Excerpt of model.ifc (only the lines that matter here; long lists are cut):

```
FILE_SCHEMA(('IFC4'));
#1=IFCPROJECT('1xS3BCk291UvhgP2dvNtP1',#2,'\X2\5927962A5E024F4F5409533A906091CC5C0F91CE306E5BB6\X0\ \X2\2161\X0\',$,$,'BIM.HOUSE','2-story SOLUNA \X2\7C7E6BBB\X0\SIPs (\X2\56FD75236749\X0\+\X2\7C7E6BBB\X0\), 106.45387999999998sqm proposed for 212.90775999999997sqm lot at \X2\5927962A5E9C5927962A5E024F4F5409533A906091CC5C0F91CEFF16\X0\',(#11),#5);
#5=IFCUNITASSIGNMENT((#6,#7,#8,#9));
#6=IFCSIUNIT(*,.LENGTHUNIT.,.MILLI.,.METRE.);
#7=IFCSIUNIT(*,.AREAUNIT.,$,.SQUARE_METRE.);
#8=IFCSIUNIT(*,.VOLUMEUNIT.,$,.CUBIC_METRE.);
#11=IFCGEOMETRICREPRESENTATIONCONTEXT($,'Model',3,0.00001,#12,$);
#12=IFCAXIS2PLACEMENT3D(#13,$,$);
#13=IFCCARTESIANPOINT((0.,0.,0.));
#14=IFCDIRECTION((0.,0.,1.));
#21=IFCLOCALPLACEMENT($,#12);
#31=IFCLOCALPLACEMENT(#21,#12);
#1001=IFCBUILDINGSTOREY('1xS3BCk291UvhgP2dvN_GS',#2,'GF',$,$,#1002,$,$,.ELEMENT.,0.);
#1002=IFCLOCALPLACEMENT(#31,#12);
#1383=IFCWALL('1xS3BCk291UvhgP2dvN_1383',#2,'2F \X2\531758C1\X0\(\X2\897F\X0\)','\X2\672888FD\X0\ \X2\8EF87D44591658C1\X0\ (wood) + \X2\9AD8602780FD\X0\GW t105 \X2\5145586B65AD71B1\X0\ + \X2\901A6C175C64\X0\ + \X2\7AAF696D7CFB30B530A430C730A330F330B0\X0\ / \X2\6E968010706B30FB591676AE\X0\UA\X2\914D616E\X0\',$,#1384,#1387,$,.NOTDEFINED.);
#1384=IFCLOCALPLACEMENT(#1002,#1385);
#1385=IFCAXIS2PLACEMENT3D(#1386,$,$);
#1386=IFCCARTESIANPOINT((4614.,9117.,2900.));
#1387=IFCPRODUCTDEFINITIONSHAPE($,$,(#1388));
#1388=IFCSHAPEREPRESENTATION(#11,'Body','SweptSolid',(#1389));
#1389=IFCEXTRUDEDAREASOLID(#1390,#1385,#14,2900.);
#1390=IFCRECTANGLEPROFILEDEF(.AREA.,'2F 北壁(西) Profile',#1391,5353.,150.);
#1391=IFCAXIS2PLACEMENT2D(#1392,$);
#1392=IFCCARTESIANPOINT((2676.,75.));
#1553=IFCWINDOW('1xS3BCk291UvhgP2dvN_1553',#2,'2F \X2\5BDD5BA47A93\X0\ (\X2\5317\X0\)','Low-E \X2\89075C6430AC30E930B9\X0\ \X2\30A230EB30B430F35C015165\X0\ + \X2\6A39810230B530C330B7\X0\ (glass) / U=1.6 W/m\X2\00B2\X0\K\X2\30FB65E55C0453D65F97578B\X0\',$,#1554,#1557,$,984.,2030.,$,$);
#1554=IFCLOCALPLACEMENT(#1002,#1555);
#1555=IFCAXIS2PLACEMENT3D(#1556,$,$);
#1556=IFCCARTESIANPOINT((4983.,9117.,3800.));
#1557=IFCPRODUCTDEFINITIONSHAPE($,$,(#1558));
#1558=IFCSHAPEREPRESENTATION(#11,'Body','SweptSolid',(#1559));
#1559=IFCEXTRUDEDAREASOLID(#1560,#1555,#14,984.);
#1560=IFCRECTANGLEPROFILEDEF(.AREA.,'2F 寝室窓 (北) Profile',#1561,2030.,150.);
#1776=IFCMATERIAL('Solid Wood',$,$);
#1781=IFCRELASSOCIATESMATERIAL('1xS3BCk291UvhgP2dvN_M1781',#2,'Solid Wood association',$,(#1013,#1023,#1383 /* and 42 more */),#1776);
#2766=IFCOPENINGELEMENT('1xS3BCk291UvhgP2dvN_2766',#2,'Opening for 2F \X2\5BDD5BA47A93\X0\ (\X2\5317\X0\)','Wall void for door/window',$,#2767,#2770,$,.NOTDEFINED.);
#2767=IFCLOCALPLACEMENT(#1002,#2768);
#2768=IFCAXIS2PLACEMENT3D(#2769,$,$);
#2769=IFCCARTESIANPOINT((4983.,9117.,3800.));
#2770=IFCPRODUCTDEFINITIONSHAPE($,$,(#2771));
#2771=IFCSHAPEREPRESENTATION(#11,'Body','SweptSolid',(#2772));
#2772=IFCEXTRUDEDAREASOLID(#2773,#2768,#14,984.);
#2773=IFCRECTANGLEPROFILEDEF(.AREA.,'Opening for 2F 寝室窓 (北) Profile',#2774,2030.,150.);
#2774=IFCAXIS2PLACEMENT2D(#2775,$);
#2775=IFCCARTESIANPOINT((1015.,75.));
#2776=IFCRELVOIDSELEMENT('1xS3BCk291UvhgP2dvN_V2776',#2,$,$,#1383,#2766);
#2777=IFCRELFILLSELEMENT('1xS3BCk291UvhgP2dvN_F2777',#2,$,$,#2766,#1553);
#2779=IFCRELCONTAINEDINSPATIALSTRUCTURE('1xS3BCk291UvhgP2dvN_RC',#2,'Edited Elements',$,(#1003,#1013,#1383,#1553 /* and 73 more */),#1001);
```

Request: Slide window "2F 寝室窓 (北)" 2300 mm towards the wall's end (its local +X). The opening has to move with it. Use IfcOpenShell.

```python
import ifcopenshell
import ifcopenshell.api.geometry
import ifcopenshell.util.placement
import ifcopenshell.util.unit

model = ifcopenshell.open("model.ifc")
unit_scale = ifcopenshell.util.unit.calculate_unit_scale(model)

window = model.by_guid("1xS3BCk291UvhgP2dvN_1553")
opening = window.FillsVoids[0].RelatingOpeningElement
wall = opening.VoidsElements[0].RelatingBuildingElement

wall_matrix = ifcopenshell.util.placement.get_local_placement(wall.ObjectPlacement)
shift = wall_matrix[:3, 0] * 2.3 / unit_scale
before = ifcopenshell.util.placement.get_local_placement(window.ObjectPlacement)[:3, 3].copy()

# The window is not placed relative to its opening, so move both.
for product in (opening, window):
    matrix = ifcopenshell.util.placement.get_local_placement(product.ObjectPlacement)
    matrix[:3, 3] += shift
    ifcopenshell.api.geometry.edit_object_placement(model, product=product, matrix=matrix, is_si=False)

after = ifcopenshell.util.placement.get_local_placement(window.ObjectPlacement)[:3, 3]
print("window moved by", (after - before).round(3) + 0.0)

model.write("model-out.ifc")
```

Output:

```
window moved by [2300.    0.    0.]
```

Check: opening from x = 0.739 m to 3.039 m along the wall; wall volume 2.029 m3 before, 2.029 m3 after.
